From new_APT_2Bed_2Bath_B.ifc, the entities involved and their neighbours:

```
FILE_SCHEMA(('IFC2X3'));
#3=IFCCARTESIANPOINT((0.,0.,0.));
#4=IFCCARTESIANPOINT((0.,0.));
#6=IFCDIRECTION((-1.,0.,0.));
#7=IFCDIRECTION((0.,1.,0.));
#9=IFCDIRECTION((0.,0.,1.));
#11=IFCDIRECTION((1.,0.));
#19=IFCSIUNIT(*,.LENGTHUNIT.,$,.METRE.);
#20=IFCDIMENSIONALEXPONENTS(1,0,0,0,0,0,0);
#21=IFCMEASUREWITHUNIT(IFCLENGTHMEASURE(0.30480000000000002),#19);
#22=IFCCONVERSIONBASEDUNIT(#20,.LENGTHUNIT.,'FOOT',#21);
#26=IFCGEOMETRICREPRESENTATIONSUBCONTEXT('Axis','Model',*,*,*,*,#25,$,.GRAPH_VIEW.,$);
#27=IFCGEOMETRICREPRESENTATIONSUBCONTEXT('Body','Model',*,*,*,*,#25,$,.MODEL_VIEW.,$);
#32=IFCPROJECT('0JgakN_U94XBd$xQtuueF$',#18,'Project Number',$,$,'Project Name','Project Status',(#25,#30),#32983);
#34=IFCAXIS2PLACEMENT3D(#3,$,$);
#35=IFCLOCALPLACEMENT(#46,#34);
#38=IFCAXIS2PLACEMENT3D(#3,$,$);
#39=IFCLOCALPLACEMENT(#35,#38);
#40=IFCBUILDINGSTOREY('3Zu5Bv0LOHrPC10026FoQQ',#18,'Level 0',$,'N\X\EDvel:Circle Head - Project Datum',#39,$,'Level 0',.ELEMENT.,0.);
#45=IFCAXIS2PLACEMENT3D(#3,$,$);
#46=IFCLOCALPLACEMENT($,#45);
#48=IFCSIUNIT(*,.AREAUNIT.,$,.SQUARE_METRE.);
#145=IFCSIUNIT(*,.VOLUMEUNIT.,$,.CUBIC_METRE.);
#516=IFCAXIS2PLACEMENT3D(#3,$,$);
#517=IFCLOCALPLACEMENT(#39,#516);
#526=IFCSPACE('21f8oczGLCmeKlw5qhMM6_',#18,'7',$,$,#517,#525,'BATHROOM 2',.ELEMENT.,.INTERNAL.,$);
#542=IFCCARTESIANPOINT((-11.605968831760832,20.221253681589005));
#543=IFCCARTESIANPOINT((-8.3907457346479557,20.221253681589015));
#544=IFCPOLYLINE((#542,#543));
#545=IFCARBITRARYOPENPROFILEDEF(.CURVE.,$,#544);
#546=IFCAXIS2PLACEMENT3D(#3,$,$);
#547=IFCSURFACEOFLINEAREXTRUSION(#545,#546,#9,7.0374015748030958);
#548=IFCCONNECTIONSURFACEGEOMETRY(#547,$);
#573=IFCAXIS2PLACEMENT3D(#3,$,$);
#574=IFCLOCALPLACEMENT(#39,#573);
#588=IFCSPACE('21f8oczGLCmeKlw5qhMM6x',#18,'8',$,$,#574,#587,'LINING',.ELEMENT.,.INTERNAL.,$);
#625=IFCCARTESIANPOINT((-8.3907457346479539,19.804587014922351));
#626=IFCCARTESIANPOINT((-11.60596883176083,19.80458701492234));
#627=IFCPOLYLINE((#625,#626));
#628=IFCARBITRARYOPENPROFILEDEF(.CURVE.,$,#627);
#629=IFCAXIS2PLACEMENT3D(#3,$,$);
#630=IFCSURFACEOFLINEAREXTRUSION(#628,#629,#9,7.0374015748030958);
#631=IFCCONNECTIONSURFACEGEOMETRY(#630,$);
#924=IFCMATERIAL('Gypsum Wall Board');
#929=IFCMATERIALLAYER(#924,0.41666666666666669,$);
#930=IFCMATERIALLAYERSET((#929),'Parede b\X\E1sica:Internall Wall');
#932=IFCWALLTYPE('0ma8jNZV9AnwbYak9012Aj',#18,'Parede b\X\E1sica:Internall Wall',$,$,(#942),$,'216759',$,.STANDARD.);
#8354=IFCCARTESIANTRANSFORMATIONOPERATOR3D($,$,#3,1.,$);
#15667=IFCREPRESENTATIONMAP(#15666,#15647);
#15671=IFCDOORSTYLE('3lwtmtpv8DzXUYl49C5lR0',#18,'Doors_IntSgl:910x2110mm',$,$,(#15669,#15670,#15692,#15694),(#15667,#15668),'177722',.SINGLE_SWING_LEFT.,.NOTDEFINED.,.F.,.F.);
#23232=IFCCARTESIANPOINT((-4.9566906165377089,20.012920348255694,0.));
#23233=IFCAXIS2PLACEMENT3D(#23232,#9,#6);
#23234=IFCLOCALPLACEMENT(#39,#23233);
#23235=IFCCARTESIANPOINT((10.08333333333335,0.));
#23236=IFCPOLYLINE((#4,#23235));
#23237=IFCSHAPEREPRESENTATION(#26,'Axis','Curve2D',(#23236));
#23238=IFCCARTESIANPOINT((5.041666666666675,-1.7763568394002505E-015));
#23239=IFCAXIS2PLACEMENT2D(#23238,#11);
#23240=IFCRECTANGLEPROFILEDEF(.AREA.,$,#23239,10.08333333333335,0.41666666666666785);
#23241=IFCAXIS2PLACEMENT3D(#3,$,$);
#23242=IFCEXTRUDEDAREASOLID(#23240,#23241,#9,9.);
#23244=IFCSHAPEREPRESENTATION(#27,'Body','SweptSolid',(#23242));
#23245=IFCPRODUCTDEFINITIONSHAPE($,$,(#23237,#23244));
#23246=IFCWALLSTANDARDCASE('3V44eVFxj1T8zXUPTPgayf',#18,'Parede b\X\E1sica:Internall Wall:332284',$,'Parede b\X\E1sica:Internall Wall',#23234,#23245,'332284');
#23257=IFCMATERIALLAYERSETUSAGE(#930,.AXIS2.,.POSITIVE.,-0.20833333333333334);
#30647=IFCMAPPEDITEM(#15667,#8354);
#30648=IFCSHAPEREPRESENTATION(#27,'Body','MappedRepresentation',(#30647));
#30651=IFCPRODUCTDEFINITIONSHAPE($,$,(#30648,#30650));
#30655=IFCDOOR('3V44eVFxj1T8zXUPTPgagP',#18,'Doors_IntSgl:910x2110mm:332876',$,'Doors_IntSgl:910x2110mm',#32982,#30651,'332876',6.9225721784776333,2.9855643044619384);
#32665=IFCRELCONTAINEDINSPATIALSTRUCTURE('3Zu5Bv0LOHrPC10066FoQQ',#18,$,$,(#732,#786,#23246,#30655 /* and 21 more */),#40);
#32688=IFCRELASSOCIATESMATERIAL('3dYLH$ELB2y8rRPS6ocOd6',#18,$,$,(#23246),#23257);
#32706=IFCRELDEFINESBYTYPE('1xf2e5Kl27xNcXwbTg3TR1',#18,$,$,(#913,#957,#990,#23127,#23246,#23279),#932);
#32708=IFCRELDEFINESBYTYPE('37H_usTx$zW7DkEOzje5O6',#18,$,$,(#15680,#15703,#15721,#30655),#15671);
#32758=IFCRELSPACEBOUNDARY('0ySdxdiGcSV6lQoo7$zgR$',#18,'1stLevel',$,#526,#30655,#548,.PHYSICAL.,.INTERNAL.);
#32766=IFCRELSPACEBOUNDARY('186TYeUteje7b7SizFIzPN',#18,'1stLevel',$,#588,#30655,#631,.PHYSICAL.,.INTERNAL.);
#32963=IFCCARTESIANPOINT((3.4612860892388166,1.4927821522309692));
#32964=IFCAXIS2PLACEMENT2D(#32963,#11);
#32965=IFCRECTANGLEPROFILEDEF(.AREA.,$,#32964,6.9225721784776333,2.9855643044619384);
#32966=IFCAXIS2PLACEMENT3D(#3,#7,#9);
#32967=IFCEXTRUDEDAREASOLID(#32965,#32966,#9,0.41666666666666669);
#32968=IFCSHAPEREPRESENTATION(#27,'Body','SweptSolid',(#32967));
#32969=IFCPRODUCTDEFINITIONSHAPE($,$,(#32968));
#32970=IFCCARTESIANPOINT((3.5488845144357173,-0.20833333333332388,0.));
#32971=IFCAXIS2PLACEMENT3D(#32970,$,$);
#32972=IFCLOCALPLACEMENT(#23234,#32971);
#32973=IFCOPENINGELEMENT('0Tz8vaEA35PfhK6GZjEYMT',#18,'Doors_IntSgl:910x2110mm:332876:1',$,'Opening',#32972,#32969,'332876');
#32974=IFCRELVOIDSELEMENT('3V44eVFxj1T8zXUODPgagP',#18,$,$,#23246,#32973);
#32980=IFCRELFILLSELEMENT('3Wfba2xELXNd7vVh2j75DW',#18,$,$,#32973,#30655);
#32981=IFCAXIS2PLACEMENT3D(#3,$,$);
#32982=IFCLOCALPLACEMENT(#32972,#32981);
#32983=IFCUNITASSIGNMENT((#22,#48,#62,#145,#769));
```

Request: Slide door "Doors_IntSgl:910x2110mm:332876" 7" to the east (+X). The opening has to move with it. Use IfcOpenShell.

```python
import numpy as np
import ifcopenshell
import ifcopenshell.api.geometry
import ifcopenshell.util.placement
import ifcopenshell.util.unit

model = ifcopenshell.open("new_APT_2Bed_2Bath_B.ifc")
unit_scale = ifcopenshell.util.unit.calculate_unit_scale(model)

door = model.by_guid("3V44eVFxj1T8zXUPTPgagP")
opening = door.FillsVoids[0].RelatingOpeningElement
wall = opening.VoidsElements[0].RelatingBuildingElement

wall_matrix = ifcopenshell.util.placement.get_local_placement(wall.ObjectPlacement)
shift = wall_matrix[:3, 0] * -7 * 0.0254 / unit_scale
before = ifcopenshell.util.placement.get_local_placement(door.ObjectPlacement)[:3, 3].copy()

# The door is placed relative to its opening, so it follows when the opening moves.
matrix = ifcopenshell.util.placement.get_local_placement(opening.ObjectPlacement)
matrix[:3, 3] += shift
ifcopenshell.api.geometry.edit_object_placement(
    model, product=opening, matrix=matrix, is_si=False, should_transform_children=True
)

# Space boundary surfaces are stored in each space's coordinates; move them too.
for rel in door.ProvidesBoundaries:
    if not rel.ConnectionGeometry:
        continue
    surface = rel.ConnectionGeometry.SurfaceOnRelatingElement
    space_matrix = ifcopenshell.util.placement.get_local_placement(rel.RelatingSpace.ObjectPlacement)
    point = np.array(surface.Position.Location.Coordinates) + space_matrix[:3, :3].T @ shift
    surface.Position = model.createIfcAxis2Placement3D(
        model.createIfcCartesianPoint(point.tolist()), surface.Position.Axis, surface.Position.RefDirection
    )

after = ifcopenshell.util.placement.get_local_placement(door.ObjectPlacement)[:3, 3]
print("door moved by", (after - before).round(3) + 0.0)

model.write("new_APT_2Bed_2Bath_B-out.ifc")
```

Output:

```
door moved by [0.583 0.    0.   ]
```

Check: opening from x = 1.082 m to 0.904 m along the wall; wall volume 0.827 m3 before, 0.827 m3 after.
